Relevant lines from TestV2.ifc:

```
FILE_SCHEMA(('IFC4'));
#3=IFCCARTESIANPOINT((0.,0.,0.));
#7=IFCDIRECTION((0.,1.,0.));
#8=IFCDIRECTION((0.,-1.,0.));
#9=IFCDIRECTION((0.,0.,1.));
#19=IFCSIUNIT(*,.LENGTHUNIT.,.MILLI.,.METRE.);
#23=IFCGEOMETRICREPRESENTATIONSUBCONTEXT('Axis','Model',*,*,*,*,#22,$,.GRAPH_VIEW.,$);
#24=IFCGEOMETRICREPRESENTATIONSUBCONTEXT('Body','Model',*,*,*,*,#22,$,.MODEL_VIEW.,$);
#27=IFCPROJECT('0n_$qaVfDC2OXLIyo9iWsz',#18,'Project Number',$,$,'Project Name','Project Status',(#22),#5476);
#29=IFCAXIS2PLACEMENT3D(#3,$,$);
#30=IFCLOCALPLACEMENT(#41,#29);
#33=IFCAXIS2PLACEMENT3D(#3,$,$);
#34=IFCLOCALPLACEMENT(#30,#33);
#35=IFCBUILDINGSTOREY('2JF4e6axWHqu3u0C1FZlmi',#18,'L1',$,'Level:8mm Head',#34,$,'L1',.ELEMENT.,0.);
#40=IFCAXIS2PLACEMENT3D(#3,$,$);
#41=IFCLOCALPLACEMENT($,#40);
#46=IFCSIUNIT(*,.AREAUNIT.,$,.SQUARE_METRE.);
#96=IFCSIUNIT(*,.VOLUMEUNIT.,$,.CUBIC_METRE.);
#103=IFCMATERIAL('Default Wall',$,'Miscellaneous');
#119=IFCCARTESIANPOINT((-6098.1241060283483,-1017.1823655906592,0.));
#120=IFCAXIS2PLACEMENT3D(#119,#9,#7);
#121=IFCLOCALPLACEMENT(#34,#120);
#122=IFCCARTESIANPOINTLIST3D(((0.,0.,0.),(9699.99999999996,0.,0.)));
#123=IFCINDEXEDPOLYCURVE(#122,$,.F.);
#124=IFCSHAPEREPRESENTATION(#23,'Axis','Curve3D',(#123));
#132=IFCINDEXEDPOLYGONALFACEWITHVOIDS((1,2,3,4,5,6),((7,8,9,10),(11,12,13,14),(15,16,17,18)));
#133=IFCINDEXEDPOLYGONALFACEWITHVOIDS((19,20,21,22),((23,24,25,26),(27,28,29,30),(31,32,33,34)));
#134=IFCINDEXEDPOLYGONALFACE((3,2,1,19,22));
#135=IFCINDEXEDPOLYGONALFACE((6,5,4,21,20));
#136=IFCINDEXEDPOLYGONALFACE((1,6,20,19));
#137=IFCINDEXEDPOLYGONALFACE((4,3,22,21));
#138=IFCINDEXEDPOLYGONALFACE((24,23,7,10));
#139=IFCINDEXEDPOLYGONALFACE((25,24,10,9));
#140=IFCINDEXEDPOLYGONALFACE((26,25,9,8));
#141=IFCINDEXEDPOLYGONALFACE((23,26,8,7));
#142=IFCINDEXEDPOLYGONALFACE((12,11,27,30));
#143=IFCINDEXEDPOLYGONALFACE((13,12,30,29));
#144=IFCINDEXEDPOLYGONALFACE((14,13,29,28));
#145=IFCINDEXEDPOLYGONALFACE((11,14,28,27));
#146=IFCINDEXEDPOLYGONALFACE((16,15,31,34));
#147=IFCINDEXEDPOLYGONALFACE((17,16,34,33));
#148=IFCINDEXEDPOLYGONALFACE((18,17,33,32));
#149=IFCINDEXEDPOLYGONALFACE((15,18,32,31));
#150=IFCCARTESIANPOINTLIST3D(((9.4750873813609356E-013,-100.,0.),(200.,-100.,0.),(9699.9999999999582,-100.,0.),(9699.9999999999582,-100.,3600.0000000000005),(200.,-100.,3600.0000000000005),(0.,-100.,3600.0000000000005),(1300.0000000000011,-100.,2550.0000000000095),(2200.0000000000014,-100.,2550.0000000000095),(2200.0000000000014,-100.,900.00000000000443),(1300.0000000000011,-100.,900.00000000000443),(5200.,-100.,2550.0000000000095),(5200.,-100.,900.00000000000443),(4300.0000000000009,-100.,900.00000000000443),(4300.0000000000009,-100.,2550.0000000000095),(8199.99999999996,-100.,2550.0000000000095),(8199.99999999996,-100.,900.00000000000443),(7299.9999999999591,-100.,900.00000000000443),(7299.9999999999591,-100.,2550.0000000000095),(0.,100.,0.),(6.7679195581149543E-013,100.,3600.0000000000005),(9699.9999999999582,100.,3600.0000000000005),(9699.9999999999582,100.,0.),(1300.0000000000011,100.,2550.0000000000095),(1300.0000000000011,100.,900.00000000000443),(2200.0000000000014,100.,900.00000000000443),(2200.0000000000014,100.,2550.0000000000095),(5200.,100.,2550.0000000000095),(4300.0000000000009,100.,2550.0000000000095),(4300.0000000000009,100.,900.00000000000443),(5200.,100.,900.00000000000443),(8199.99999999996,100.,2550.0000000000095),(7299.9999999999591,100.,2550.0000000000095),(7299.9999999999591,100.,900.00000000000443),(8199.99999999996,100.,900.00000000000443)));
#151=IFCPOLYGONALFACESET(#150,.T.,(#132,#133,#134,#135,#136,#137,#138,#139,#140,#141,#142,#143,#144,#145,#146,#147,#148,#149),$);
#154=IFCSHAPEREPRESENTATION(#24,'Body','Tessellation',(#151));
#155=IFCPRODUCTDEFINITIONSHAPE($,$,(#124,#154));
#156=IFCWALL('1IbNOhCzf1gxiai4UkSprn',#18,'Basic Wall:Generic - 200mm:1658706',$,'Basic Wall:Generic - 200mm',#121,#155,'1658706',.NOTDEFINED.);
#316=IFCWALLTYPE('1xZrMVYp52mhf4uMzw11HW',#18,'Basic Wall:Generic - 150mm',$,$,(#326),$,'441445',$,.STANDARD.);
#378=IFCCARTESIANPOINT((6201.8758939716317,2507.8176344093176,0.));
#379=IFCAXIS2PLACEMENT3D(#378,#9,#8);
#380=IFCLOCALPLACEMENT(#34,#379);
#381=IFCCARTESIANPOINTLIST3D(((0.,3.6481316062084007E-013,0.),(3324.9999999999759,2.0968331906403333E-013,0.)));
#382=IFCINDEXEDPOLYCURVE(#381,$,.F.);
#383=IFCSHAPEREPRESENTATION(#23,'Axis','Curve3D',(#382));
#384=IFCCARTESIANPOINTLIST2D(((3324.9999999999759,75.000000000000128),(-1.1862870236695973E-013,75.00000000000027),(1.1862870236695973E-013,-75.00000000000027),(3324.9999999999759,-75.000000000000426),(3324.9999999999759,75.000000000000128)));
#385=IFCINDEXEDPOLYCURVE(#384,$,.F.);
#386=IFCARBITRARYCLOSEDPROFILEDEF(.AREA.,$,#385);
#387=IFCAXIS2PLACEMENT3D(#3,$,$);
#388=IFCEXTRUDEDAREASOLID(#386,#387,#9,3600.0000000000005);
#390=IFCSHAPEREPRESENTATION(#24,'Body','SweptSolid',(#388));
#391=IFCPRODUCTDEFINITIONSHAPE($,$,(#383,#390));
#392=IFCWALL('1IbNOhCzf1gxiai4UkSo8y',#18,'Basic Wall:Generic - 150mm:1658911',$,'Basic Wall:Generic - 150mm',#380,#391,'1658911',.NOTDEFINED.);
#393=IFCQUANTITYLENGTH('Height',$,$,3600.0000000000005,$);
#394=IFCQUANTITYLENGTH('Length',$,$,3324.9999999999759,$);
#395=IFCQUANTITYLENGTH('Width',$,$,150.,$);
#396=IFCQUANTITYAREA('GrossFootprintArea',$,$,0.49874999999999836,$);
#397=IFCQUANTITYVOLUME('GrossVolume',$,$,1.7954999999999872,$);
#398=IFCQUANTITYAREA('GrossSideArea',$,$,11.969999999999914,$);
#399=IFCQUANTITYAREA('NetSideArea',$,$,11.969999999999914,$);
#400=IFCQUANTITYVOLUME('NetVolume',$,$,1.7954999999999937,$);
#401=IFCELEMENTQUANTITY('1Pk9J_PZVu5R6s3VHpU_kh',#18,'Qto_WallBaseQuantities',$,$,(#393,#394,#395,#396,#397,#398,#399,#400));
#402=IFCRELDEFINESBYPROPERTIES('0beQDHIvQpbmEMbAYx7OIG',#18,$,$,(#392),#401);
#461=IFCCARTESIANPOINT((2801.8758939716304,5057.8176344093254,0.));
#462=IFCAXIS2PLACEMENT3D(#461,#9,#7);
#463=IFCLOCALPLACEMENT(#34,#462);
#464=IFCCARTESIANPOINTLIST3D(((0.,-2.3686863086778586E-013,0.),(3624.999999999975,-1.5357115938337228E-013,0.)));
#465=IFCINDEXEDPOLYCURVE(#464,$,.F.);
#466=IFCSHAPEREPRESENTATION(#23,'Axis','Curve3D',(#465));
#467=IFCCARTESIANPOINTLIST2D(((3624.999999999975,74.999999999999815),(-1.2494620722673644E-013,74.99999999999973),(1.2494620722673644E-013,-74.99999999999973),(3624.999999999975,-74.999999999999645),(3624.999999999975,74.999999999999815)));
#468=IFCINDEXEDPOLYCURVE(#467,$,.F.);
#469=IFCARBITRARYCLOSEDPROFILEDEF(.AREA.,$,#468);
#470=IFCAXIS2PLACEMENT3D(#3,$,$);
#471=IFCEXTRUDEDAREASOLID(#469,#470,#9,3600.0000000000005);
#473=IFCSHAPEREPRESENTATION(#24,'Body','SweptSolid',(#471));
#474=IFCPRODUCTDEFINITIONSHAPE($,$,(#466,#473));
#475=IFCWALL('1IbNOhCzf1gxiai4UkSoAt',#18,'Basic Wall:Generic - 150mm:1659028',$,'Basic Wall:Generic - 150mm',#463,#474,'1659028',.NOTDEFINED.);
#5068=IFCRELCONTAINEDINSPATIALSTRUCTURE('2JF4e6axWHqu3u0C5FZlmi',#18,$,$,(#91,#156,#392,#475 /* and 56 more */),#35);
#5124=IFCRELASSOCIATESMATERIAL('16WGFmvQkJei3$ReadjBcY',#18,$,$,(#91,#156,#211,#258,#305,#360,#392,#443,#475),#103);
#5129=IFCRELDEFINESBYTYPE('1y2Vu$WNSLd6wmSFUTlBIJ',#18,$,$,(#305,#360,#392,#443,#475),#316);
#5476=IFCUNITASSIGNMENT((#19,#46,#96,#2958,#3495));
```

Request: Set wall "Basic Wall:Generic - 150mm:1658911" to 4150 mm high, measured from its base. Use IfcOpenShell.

```python
import ifcopenshell
import ifcopenshell.api.pset
import ifcopenshell.geom
import ifcopenshell.util.element
import ifcopenshell.util.representation
import ifcopenshell.util.shape
import ifcopenshell.util.unit

model = ifcopenshell.open("TestV2.ifc")
unit_scale = ifcopenshell.util.unit.calculate_unit_scale(model)
area_scale = ifcopenshell.util.unit.calculate_unit_scale(model, "AREAUNIT")
volume_scale = ifcopenshell.util.unit.calculate_unit_scale(model, "VOLUMEUNIT")
settings = ifcopenshell.geom.settings()


def volume(element):
    """Net volume in cubic metres, openings subtracted."""
    shape = ifcopenshell.geom.create_shape(settings, element)
    return ifcopenshell.util.shape.get_volume(shape.geometry)


wall = model.by_guid("1IbNOhCzf1gxiai4UkSo8y")
before = volume(wall)

body = ifcopenshell.util.representation.get_representation(wall, "Model", "Body")
solid = body.Items[0]
old_height = solid.Depth
solid.Depth = 4150.0
after = volume(wall)
thickness = 0.15  # wall thickness in metres

# Update the stored height, areas and volumes.
qto = model.by_id(ifcopenshell.util.element.get_pset(wall, "Qto_WallBaseQuantities", should_inherit=False)["id"])
ifcopenshell.api.pset.edit_qto(model, qto=qto, properties={
    "Height": solid.Depth,
    "GrossVolume": ifcopenshell.util.element.get_pset(wall, "Qto_WallBaseQuantities", "GrossVolume") * solid.Depth / old_height,
    "GrossSideArea": ifcopenshell.util.element.get_pset(wall, "Qto_WallBaseQuantities", "GrossSideArea") * solid.Depth / old_height,
    "NetSideArea": after / thickness / area_scale,
    "NetVolume": after / volume_scale,
})

print(f"height {old_height:g} -> {solid.Depth:g}, volume {before:.3f} -> {after:.3f} m3")

model.write("TestV2_edited.ifc")
```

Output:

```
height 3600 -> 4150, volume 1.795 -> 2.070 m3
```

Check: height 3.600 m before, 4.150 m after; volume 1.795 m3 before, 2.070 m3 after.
